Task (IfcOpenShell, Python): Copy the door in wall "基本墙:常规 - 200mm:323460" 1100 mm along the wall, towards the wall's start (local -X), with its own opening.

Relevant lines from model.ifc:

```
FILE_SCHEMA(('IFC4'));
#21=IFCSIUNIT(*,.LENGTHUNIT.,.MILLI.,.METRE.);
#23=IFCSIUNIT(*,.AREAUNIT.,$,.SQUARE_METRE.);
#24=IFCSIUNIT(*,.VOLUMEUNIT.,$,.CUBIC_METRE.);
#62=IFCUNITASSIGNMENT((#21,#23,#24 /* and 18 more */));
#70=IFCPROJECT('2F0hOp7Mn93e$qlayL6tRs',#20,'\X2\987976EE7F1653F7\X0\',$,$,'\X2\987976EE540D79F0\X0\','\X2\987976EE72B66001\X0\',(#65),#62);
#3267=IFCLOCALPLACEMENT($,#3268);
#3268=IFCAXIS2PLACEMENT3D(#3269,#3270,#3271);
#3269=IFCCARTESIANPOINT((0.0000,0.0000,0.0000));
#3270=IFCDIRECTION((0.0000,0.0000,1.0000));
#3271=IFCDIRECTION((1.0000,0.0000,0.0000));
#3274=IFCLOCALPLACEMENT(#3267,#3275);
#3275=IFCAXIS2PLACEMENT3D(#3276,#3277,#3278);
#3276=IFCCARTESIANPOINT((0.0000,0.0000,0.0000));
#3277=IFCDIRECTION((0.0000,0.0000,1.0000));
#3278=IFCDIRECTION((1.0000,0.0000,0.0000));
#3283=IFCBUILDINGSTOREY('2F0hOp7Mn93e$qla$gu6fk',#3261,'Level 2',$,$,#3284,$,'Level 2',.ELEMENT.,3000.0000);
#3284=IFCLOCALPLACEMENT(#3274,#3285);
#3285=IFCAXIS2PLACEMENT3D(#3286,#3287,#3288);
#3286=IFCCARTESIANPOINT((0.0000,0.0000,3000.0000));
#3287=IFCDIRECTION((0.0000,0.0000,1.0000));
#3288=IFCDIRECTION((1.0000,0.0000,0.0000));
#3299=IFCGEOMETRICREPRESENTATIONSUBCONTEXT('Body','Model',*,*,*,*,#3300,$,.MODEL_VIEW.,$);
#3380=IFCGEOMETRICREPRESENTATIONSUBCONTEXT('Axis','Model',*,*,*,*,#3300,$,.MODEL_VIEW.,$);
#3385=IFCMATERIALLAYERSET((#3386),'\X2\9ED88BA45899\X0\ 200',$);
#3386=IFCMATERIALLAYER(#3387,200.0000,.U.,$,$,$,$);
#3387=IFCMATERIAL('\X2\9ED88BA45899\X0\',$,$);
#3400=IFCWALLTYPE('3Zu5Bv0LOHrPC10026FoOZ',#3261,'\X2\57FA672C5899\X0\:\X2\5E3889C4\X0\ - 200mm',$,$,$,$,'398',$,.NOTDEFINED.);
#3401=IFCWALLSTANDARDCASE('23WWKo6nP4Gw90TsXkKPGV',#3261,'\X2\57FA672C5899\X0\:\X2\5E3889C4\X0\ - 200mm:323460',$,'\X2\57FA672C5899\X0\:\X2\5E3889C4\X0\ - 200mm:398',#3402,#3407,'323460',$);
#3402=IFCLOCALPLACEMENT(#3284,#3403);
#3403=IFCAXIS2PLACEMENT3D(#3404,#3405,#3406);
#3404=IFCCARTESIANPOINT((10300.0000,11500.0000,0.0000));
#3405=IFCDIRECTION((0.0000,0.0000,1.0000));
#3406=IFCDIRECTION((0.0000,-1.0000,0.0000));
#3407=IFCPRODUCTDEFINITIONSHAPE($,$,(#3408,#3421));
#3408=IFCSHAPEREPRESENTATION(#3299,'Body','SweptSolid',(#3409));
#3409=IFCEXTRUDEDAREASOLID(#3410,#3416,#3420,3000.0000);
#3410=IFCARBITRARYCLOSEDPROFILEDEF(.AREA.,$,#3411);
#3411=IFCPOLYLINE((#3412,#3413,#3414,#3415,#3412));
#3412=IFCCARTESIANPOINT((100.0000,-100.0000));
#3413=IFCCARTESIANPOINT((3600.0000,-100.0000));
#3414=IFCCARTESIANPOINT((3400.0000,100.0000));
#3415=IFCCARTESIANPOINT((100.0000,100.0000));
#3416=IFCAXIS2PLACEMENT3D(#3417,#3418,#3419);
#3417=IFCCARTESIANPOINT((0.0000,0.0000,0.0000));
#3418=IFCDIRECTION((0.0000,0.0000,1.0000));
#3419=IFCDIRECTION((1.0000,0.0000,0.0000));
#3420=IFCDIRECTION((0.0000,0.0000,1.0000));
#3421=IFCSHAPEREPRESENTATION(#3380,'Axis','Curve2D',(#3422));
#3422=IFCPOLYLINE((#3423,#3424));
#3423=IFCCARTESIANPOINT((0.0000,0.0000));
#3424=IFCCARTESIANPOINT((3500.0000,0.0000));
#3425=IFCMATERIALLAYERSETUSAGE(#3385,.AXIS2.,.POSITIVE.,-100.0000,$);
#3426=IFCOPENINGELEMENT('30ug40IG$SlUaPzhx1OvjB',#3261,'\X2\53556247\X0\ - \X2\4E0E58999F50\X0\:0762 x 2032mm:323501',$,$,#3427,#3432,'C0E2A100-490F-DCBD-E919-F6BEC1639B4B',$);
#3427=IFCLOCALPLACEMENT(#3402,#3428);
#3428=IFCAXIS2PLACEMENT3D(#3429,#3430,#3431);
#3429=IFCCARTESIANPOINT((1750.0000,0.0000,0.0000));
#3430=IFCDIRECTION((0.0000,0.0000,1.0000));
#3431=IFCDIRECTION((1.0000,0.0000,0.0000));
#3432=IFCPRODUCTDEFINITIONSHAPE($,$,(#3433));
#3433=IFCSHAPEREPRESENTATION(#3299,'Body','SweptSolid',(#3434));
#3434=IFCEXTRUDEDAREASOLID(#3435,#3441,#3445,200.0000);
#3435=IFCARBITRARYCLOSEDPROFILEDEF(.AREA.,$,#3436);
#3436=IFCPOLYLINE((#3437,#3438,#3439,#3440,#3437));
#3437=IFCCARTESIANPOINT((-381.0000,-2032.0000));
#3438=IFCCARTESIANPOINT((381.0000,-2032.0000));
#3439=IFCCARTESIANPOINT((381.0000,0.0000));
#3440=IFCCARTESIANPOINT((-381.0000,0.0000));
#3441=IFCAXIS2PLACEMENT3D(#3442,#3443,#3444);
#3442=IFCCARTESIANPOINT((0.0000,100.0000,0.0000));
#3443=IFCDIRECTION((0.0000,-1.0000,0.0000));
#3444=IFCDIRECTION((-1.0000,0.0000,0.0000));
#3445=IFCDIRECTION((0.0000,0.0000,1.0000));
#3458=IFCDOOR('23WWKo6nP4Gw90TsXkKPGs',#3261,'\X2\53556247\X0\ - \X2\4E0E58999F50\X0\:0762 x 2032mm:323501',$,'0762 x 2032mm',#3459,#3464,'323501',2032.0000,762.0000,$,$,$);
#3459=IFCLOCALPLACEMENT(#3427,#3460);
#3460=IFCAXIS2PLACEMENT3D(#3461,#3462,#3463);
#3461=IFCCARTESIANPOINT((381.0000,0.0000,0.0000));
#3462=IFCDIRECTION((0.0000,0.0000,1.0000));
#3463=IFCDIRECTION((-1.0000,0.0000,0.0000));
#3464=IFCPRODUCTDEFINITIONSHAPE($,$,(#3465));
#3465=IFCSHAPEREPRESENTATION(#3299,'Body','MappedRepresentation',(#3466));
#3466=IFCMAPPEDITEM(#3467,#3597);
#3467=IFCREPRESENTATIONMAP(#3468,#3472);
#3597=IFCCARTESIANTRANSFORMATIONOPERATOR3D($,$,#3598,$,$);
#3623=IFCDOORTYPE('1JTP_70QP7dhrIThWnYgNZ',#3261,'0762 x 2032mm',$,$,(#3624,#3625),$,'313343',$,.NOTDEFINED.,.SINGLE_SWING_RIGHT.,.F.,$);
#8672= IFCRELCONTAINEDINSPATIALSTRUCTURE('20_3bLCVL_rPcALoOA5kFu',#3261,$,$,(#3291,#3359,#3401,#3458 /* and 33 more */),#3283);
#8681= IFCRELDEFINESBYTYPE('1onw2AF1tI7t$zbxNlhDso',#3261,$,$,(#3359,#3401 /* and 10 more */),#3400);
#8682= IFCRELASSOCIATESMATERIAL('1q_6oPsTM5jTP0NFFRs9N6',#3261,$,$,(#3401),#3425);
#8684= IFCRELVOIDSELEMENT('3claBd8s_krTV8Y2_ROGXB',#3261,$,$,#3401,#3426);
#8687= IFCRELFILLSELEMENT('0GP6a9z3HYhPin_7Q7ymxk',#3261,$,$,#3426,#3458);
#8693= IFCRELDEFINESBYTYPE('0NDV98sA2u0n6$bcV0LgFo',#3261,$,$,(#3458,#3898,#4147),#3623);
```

```python
import ifcopenshell
import ifcopenshell.api.feature
import ifcopenshell.api.geometry
import ifcopenshell.api.root
import ifcopenshell.geom
import ifcopenshell.util.element
import ifcopenshell.util.placement
import ifcopenshell.util.shape
import ifcopenshell.util.unit

model = ifcopenshell.open("model.ifc")
unit_scale = ifcopenshell.util.unit.calculate_unit_scale(model)
settings = ifcopenshell.geom.settings()


def volume(element):
    """Net volume in cubic metres, openings subtracted."""
    shape = ifcopenshell.geom.create_shape(settings, element)
    return ifcopenshell.util.shape.get_volume(shape.geometry)


def reuse_history(source, copy):
    """copy_class also copies each property set's owner history, people and application; keep the originals."""
    for rel in copy.IsDefinedBy:
        if rel.is_a("IfcRelDefinesByProperties") and (history := rel.RelatingPropertyDefinition.OwnerHistory):
            rel.RelatingPropertyDefinition.OwnerHistory = source.OwnerHistory
            ifcopenshell.util.element.remove_deep2(model, history)


door = model.by_id(3458)
opening = door.FillsVoids[0].RelatingOpeningElement
wall = opening.VoidsElements[0].RelatingBuildingElement
before = volume(wall)
shift = ifcopenshell.util.placement.get_local_placement(wall.ObjectPlacement)[:3, 0] * -1.1 / unit_scale

# copy_class copies the void relationship, type, container and properties, but no geometry.
new_opening = ifcopenshell.api.root.copy_class(model, product=opening)
new_opening.Representation = ifcopenshell.util.element.copy_deep(
    model, opening.Representation, exclude=["IfcGeometricRepresentationContext", "IfcRepresentationMap"]
)
new_opening.Name = "单扇 - 与墙齐:0762 x 2032mm"
new_opening.Tag = None
new_door = ifcopenshell.api.root.copy_class(model, product=door)
new_door.Representation = ifcopenshell.util.element.copy_deep(
    model, door.Representation, exclude=["IfcGeometricRepresentationContext", "IfcRepresentationMap"]
)
new_door.Name = "单扇 - 与墙齐:0762 x 2032mm"
new_door.Tag = None
reuse_history(door, new_door)
ifcopenshell.api.feature.add_filling(model, opening=new_opening, element=new_door)

for old, new in ((opening, new_opening), (door, new_door)):
    matrix = ifcopenshell.util.placement.get_local_placement(old.ObjectPlacement)
    matrix[:3, 3] += shift
    ifcopenshell.api.geometry.edit_object_placement(model, product=new, matrix=matrix, is_si=False)

after = volume(wall)

print(f"wall volume {before:.3f} -> {after:.3f} m3")

model.write("model_v2.ifc")
```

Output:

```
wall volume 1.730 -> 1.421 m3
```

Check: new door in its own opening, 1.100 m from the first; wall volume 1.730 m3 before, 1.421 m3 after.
